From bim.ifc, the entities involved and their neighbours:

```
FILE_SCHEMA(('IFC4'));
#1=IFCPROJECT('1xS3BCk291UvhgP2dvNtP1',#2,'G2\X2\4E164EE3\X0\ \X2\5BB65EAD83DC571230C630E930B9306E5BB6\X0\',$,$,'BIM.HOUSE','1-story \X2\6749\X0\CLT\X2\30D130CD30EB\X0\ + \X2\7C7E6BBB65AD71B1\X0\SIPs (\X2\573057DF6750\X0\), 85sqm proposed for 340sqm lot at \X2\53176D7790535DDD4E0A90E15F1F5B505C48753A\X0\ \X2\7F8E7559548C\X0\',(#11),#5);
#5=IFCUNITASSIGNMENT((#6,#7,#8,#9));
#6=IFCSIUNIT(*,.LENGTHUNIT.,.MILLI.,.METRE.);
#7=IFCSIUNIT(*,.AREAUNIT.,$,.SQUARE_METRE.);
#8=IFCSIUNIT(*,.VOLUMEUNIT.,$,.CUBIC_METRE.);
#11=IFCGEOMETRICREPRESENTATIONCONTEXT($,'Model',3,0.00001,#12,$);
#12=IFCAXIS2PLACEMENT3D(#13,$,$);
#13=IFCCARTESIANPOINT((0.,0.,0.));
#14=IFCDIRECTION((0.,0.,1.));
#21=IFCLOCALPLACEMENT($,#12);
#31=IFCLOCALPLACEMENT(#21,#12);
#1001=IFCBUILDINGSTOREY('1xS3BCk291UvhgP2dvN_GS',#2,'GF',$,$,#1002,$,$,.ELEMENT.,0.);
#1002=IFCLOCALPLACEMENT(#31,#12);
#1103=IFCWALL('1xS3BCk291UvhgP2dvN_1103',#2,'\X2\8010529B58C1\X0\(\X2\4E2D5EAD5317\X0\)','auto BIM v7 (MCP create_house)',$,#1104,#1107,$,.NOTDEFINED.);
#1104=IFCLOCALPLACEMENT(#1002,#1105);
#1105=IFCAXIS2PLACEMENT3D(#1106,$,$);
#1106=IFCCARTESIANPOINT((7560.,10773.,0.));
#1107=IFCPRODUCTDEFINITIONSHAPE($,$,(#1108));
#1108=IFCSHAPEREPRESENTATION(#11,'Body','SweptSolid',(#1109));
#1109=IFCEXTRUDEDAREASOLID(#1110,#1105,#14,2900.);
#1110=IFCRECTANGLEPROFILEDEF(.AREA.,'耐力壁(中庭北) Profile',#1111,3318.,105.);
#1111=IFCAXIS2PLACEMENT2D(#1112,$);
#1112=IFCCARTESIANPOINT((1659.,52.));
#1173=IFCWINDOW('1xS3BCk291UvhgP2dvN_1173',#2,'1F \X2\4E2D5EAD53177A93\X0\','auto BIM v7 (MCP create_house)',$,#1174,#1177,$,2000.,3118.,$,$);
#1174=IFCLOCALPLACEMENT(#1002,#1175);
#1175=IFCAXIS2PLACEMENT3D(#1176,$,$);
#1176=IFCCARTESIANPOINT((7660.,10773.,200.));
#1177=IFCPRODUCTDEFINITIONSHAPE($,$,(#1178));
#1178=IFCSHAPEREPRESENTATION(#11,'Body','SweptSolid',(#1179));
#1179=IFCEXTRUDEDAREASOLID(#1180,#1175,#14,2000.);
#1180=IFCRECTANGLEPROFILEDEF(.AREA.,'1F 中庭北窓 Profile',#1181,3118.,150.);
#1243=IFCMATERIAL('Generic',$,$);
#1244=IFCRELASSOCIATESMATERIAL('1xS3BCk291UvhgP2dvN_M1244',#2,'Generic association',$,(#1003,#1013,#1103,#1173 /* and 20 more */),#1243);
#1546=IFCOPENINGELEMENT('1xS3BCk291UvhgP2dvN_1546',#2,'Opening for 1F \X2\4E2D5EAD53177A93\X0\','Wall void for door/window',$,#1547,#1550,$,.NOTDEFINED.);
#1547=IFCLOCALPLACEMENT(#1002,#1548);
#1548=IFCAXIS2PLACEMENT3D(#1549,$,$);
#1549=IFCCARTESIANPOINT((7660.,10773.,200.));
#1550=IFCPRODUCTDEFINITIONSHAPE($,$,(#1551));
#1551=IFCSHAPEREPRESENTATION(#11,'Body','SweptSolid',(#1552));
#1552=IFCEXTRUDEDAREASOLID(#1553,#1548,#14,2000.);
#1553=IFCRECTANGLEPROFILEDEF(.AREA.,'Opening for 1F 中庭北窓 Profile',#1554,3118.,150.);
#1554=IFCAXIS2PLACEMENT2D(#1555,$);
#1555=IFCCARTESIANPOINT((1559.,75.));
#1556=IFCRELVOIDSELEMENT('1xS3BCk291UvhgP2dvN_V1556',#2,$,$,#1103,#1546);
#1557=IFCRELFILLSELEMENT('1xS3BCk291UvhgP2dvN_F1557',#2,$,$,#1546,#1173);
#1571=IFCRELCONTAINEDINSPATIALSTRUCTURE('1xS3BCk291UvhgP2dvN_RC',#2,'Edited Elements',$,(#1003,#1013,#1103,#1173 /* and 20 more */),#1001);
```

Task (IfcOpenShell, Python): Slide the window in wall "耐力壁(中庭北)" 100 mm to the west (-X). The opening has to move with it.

```python
import ifcopenshell
import ifcopenshell.api.geometry
import ifcopenshell.util.placement

model = ifcopenshell.open("bim.ifc")

window = model.by_guid("1xS3BCk291UvhgP2dvN_1173")
opening = window.FillsVoids[0].RelatingOpeningElement
wall = opening.VoidsElements[0].RelatingBuildingElement

wall_matrix = ifcopenshell.util.placement.get_local_placement(wall.ObjectPlacement)
shift = wall_matrix[:3, 0] * -100.0
before = ifcopenshell.util.placement.get_local_placement(window.ObjectPlacement)[:3, 3].copy()

# The window is not placed relative to its opening, so move both.
for product in (opening, window):
    matrix = ifcopenshell.util.placement.get_local_placement(product.ObjectPlacement)
    matrix[:3, 3] += shift
    ifcopenshell.api.geometry.edit_object_placement(model, product=product, matrix=matrix, is_si=False)

after = ifcopenshell.util.placement.get_local_placement(window.ObjectPlacement)[:3, 3]
print("window moved by", (after - before).round(3) + 0.0)

model.write("bim_rev.ifc")
```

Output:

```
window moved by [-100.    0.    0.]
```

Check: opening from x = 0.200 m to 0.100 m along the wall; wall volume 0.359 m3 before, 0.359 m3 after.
